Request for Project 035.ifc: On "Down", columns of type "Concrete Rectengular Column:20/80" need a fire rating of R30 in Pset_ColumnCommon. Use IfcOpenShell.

First a look at what the model holds.

```python
import ifcopenshell
import ifcopenshell.util.element

model = ifcopenshell.open("Project 035.ifc")
print(model.schema)
storey = next(s for s in model.by_type("IfcBuildingStorey") if s.Name == "Down")
columns = [e for e in ifcopenshell.util.element.get_decomposition(storey) if e.is_a("IfcColumn")]
seen = {}
for e in columns:
    element_type = ifcopenshell.util.element.get_type(e)
    key = (element_type.Name if element_type != e and element_type else None, ifcopenshell.util.element.get_pset(e, "Pset_ColumnCommon", "FireRating"))
    seen[key] = seen.get(key, 0) + 1
for (name, value), count in sorted(seen.items(), key=str):
    print(count, "x", name, "|", value)
```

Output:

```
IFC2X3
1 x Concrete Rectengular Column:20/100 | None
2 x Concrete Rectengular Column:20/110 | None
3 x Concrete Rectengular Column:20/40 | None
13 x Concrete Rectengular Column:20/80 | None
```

```python
import ifcopenshell
import ifcopenshell.api.pset
import ifcopenshell.util.element

model = ifcopenshell.open("Project 035.ifc")

storey = next(s for s in model.by_type("IfcBuildingStorey") if s.Name == "Down")
columns = [e for e in ifcopenshell.util.element.get_decomposition(storey) if e.is_a("IfcColumn")]

count = 0
for e in columns:
    element_type = ifcopenshell.util.element.get_type(e)
    if element_type in (None, e) or element_type.Name != "Concrete Rectengular Column:20/80":
        continue
    # add_pset returns the element's existing set when there is one.
    pset = ifcopenshell.api.pset.add_pset(model, product=e, name="Pset_ColumnCommon")
    ifcopenshell.api.pset.edit_pset(model, pset=pset, properties={"FireRating": "R30"})
    count += 1

print(count, "columns updated")

model.write("Project 035_updated.ifc")
```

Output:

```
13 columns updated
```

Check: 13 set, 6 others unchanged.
